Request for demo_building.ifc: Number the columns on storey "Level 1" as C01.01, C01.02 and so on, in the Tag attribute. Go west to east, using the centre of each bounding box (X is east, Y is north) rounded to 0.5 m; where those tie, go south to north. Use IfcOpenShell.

First a look at what the model holds.

```python
import ifcopenshell
import ifcopenshell.util.element
import ifcopenshell.util.placement

model = ifcopenshell.open("demo_building.ifc")
print(model.schema)
storey = next(s for s in model.by_type("IfcBuildingStorey") if s.Name == "Level 1")
columns = [e for e in ifcopenshell.util.element.get_decomposition(storey) if e.is_a("IfcColumn")]
for e in sorted(columns, key=lambda e: e.id()):
    origin = ifcopenshell.util.placement.get_local_placement(e.ObjectPlacement)[:3, 3]
    print(e.id(), e.Tag, e.Name, origin.round(2) + 0.0, sep=" | ")
```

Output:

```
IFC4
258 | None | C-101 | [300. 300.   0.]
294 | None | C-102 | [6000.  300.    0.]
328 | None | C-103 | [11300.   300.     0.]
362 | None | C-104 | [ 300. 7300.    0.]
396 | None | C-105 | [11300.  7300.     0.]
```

```python
import ifcopenshell
import ifcopenshell.geom
import ifcopenshell.util.element
import ifcopenshell.util.shape

model = ifcopenshell.open("demo_building.ifc")
settings = ifcopenshell.geom.settings()
settings.set("use-world-coords", True)


def centre(element):
    shape = ifcopenshell.geom.create_shape(settings, element)
    return ifcopenshell.util.shape.get_bbox_centroid(shape.geometry)


storey = next(s for s in model.by_type("IfcBuildingStorey") if s.Name == "Level 1")
columns = [e for e in ifcopenshell.util.element.get_decomposition(storey) if e.is_a("IfcColumn")]

# Insertion points can sit at a corner or the storey origin, so sort by the geometry (in metres).
centres = {e: centre(e) for e in columns}
columns.sort(key=lambda e: (round(centres[e][0] / 0.5), centres[e][1]))

for i, e in enumerate(columns, start=1):
    number = f"C01.{i:02d}"
    e.Tag = number
    print(e.id(), number)

model.write("demo_building_v2.ifc")
```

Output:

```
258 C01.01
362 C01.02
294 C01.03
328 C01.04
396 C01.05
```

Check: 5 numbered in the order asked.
